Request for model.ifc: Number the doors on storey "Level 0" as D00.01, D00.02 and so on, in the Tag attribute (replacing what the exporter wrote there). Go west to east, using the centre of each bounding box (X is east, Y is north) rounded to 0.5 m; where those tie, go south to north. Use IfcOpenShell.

First a look at what the model holds.

```python
import ifcopenshell
import ifcopenshell.util.element
import ifcopenshell.util.placement

model = ifcopenshell.open("model.ifc")
print(model.schema)
storey = next(s for s in model.by_type("IfcBuildingStorey") if s.Name == "Level 0")
doors = [e for e in ifcopenshell.util.element.get_decomposition(storey) if e.is_a("IfcDoor")]
for e in sorted(doors, key=lambda e: e.id()):
    origin = ifcopenshell.util.placement.get_local_placement(e.ObjectPlacement)[:3, 3]
    print(e.id(), e.Tag, e.Name, origin.round(2) + 0.0, sep=" | ")
```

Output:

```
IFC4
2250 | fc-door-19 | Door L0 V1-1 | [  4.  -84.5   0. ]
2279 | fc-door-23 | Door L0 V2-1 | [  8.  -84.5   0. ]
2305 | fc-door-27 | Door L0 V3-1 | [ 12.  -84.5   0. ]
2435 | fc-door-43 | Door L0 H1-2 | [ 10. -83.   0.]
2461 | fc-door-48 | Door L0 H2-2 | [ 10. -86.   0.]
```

```python
import ifcopenshell
import ifcopenshell.geom
import ifcopenshell.util.element
import ifcopenshell.util.shape

model = ifcopenshell.open("model.ifc")
settings = ifcopenshell.geom.settings()
settings.set("use-world-coords", True)


def centre(element):
    shape = ifcopenshell.geom.create_shape(settings, element)
    return ifcopenshell.util.shape.get_bbox_centroid(shape.geometry)


storey = next(s for s in model.by_type("IfcBuildingStorey") if s.Name == "Level 0")
doors = [e for e in ifcopenshell.util.element.get_decomposition(storey) if e.is_a("IfcDoor")]

# Insertion points can sit at a corner or the storey origin, so sort by the geometry (in metres).
centres = {e: centre(e) for e in doors}
doors.sort(key=lambda e: (round(centres[e][0] / 0.5), centres[e][1]))

for i, e in enumerate(doors, start=1):
    number = f"D00.{i:02d}"
    e.Tag = number
    print(e.id(), number)

model.write("model_v2.ifc")
```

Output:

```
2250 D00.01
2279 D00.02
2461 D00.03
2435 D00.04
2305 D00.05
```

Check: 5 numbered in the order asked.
